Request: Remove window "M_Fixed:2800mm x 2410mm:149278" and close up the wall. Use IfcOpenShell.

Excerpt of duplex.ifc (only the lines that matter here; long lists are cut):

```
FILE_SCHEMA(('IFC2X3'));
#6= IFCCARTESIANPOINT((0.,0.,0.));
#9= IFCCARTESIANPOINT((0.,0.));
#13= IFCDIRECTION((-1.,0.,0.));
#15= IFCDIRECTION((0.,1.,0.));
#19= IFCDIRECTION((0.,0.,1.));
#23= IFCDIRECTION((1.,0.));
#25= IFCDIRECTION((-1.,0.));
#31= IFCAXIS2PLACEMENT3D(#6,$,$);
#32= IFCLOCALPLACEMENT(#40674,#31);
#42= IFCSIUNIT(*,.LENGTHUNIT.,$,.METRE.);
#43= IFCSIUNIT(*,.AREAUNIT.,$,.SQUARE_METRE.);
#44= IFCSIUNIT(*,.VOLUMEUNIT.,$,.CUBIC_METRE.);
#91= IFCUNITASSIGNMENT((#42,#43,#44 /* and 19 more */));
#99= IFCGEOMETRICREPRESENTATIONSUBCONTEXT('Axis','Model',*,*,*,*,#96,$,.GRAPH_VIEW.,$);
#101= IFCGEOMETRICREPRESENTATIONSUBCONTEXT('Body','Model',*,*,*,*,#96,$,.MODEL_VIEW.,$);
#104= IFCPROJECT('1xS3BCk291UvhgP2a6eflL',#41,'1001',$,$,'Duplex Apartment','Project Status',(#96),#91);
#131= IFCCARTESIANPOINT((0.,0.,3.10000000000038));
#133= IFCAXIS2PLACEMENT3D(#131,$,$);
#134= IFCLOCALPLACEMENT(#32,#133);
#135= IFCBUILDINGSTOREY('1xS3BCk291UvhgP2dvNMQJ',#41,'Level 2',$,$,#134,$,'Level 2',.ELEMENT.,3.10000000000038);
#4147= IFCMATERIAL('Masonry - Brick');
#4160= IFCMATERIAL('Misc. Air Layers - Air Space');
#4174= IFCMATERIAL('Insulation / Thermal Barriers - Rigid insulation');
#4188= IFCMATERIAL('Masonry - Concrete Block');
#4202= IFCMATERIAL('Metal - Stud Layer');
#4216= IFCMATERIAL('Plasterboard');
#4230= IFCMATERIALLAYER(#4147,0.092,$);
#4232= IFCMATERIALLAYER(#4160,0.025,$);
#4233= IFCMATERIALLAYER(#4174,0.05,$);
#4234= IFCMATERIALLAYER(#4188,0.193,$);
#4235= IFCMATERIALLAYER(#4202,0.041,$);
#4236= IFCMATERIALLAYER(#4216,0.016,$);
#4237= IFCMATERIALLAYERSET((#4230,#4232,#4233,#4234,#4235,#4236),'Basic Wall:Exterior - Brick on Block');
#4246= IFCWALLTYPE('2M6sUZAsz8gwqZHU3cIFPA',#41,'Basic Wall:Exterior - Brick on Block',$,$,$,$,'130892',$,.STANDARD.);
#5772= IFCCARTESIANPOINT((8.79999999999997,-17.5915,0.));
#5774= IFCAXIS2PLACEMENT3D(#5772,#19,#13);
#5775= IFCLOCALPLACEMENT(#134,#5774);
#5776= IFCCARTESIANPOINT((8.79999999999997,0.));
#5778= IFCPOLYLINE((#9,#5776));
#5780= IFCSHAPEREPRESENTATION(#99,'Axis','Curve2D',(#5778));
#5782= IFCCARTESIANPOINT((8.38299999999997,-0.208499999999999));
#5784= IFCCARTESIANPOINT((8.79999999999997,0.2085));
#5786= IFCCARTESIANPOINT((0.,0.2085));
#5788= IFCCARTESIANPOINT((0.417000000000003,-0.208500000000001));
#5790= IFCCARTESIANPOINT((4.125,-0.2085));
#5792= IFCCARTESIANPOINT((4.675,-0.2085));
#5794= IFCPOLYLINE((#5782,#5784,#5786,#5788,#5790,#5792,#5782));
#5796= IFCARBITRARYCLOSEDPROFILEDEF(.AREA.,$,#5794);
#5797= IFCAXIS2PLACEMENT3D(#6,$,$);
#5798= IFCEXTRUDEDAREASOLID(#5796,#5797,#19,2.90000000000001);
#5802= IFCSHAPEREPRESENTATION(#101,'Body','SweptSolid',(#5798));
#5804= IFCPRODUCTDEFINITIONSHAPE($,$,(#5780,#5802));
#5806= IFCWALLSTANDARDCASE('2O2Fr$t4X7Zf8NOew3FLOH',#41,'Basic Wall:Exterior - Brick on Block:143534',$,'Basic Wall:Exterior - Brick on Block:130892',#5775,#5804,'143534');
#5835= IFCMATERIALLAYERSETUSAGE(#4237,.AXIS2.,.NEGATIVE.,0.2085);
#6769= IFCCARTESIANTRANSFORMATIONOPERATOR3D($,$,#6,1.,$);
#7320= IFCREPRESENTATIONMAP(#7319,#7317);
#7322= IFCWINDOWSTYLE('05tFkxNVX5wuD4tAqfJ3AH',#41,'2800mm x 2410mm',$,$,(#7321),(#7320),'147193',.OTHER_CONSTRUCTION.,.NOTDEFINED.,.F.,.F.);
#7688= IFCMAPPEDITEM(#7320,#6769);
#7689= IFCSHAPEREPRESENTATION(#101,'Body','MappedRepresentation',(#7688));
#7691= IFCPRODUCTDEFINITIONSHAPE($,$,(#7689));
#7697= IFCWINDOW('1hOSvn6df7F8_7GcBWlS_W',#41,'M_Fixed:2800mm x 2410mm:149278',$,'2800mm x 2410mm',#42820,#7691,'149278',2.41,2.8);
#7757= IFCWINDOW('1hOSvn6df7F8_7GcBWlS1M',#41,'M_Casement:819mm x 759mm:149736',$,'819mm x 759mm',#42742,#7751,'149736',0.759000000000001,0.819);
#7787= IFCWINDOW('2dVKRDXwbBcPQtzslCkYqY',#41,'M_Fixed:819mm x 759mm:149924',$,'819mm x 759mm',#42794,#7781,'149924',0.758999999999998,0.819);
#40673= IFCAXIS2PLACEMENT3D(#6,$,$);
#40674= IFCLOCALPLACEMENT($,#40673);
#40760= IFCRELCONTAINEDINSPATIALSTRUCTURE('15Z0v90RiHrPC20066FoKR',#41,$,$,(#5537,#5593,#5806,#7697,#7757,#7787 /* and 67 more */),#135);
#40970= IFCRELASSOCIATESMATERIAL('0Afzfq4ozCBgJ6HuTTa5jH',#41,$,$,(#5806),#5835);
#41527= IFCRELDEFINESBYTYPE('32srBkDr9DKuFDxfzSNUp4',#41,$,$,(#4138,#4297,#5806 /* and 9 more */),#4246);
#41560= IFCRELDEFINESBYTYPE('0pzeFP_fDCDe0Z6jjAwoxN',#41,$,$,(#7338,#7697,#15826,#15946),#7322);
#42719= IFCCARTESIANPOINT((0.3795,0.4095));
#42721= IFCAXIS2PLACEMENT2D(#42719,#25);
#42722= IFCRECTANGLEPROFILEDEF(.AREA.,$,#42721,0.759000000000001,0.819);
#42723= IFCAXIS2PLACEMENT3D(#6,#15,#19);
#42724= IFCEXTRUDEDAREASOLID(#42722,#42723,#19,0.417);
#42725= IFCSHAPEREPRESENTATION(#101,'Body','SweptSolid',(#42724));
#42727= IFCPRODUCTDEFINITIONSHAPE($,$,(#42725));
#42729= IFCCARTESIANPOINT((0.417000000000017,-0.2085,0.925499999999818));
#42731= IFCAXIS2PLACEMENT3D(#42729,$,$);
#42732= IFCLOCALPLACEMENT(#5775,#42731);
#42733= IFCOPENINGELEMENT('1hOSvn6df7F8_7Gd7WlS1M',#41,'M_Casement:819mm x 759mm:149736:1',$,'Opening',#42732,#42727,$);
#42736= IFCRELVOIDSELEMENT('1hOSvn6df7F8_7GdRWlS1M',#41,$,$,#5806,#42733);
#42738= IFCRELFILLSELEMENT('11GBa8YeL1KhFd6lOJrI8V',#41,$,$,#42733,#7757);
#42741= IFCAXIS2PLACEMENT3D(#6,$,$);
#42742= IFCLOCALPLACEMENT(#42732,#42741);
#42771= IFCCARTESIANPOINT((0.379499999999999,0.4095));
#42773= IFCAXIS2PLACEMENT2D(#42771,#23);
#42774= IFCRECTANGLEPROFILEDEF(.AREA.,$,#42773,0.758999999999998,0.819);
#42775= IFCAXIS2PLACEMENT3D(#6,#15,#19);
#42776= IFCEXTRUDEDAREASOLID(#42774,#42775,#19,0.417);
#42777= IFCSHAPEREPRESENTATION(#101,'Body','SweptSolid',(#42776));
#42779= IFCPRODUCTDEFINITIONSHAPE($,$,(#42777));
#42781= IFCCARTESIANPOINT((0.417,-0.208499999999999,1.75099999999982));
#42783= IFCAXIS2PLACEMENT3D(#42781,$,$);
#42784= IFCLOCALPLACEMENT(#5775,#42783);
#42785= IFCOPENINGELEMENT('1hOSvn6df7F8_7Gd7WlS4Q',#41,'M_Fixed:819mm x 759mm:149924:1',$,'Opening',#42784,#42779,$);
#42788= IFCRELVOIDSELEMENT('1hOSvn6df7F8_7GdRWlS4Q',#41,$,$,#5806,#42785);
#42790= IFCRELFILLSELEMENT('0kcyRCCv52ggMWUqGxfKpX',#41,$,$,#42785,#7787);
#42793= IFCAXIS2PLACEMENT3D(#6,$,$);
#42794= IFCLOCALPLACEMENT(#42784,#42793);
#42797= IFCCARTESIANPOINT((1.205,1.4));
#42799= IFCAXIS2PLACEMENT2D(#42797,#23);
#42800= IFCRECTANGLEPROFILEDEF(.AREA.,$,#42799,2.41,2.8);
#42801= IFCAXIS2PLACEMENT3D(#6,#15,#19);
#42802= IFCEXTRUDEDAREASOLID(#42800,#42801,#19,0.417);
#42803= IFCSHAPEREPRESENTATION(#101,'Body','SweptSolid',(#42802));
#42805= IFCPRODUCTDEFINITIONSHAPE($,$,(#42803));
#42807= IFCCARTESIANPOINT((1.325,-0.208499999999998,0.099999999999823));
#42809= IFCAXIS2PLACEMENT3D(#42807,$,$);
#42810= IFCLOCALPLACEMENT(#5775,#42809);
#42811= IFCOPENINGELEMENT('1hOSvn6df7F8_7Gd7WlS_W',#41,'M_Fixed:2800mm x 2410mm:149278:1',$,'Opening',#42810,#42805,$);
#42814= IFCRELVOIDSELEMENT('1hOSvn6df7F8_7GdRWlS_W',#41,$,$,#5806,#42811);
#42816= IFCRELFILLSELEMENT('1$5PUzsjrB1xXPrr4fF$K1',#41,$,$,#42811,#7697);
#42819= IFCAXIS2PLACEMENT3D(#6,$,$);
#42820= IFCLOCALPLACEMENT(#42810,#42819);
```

```python
import ifcopenshell
import ifcopenshell.api.feature
import ifcopenshell.api.root
import ifcopenshell.geom
import ifcopenshell.util.shape

model = ifcopenshell.open("duplex.ifc")
settings = ifcopenshell.geom.settings()


def volume(element):
    """Net volume in cubic metres, openings subtracted."""
    shape = ifcopenshell.geom.create_shape(settings, element)
    return ifcopenshell.util.shape.get_volume(shape.geometry)


window = model.by_id(7697)
opening = window.FillsVoids[0].RelatingOpeningElement
wall = opening.VoidsElements[0].RelatingBuildingElement
before = volume(wall)

ifcopenshell.api.root.remove_product(model, product=window)
ifcopenshell.api.feature.remove_feature(model, feature=opening)

after = volume(wall)

print(f"wall volume {before:.3f} -> {after:.3f} m3")

model.write("duplex_updated.ifc")
```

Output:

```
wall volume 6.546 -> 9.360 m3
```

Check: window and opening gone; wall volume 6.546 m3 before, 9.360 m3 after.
